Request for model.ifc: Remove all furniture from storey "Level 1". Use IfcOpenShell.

First a look at what the model holds.

```python
import ifcopenshell
import ifcopenshell.util.element

model = ifcopenshell.open("model.ifc")
print(model.schema)
storey = next(s for s in model.by_type("IfcBuildingStorey") if s.Name == "Level 1")
furniture = [e for e in ifcopenshell.util.element.get_decomposition(storey) if e.is_a("IfcFurnishingElement")]
seen = {}
for e in furniture:
    element_type = ifcopenshell.util.element.get_type(e)
    name = element_type.Name if element_type not in (None, e) else None
    seen[name] = seen.get(name, 0) + 1
for name, count in sorted(seen.items(), key=str):
    print(count, "x", name)
```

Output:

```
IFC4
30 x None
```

```python
import ifcopenshell
import ifcopenshell.api.root
import ifcopenshell.util.element

model = ifcopenshell.open("model.ifc")

storey = next(s for s in model.by_type("IfcBuildingStorey") if s.Name == "Level 1")
furniture = [e for e in ifcopenshell.util.element.get_decomposition(storey) if e.is_a("IfcFurnishingElement")]

for e in furniture:
    ifcopenshell.api.root.remove_product(model, product=e)
print(len(furniture), "removed")

model.write("model_rev.ifc")
```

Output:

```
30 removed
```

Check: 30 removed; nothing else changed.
